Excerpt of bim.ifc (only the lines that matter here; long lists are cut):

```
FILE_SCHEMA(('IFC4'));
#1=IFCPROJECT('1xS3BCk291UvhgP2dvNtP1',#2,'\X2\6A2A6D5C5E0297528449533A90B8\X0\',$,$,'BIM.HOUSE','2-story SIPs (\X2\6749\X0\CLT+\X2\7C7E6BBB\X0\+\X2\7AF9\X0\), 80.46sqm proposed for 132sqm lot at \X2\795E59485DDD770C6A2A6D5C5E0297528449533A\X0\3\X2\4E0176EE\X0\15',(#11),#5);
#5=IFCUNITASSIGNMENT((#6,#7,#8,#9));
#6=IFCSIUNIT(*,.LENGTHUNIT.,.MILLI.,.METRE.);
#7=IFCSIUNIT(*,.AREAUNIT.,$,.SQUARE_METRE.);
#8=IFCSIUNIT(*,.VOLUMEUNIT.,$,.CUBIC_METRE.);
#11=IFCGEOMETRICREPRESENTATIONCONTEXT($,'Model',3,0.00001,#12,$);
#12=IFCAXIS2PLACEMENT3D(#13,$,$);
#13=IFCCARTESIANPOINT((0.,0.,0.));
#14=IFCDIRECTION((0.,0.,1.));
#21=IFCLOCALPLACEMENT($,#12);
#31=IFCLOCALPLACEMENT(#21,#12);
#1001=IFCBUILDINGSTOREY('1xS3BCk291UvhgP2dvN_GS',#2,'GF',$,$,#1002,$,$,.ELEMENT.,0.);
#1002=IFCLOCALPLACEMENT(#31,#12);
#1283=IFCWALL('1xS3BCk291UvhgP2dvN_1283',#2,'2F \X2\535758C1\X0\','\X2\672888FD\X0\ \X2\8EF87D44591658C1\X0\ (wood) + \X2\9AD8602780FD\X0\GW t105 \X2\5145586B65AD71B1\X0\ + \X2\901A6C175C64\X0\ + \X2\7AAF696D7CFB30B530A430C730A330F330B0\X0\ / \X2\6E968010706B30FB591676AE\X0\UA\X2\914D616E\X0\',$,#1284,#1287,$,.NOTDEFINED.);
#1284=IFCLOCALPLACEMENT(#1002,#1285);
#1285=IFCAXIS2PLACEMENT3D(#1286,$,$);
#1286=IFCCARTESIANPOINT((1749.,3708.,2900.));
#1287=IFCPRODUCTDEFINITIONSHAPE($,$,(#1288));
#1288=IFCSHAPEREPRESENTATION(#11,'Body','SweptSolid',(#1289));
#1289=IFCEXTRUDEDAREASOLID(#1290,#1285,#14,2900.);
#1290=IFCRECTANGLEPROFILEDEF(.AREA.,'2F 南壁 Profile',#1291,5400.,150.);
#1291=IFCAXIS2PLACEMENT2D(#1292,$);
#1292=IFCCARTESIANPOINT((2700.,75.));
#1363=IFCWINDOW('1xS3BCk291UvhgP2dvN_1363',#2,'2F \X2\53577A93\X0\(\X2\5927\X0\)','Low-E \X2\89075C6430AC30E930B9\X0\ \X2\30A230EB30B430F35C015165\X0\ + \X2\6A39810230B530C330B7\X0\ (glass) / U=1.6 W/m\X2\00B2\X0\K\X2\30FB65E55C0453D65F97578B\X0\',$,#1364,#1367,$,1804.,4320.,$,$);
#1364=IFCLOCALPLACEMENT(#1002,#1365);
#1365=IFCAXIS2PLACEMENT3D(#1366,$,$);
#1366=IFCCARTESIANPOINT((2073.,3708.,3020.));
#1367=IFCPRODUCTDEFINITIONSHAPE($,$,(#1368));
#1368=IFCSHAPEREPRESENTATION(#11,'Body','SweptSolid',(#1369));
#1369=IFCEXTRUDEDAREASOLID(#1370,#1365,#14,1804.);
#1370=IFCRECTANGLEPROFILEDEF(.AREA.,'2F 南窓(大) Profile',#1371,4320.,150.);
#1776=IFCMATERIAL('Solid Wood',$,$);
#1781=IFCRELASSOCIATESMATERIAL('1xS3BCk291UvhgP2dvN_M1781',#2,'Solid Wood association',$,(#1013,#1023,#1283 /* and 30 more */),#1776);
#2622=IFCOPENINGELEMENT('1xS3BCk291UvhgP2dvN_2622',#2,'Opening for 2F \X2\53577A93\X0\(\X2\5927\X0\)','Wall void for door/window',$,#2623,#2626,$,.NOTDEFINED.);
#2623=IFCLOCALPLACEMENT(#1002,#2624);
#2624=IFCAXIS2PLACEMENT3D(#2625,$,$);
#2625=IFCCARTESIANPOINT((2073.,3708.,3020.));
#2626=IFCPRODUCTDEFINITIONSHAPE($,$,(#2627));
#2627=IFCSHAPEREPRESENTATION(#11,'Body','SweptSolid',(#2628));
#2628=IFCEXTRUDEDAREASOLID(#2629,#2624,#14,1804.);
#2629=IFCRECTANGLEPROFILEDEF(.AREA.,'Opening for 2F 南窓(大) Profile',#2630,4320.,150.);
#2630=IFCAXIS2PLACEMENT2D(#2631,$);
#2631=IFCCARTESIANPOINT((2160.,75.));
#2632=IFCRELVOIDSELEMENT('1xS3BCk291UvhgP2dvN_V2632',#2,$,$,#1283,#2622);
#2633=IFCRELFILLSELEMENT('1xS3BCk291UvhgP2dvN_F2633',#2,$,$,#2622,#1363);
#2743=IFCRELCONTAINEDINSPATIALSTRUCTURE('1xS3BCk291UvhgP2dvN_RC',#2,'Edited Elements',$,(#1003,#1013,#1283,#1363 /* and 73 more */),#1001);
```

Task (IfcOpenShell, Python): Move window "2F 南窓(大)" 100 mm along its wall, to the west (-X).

```python
import ifcopenshell
import ifcopenshell.api.geometry
import ifcopenshell.util.placement

model = ifcopenshell.open("bim.ifc")

window = model.by_guid("1xS3BCk291UvhgP2dvN_1363")
opening = window.FillsVoids[0].RelatingOpeningElement
wall = opening.VoidsElements[0].RelatingBuildingElement

wall_matrix = ifcopenshell.util.placement.get_local_placement(wall.ObjectPlacement)
shift = wall_matrix[:3, 0] * -100.0
before = ifcopenshell.util.placement.get_local_placement(window.ObjectPlacement)[:3, 3].copy()

# The window is not placed relative to its opening, so move both.
for product in (opening, window):
    matrix = ifcopenshell.util.placement.get_local_placement(product.ObjectPlacement)
    matrix[:3, 3] += shift
    ifcopenshell.api.geometry.edit_object_placement(model, product=product, matrix=matrix, is_si=False)

after = ifcopenshell.util.placement.get_local_placement(window.ObjectPlacement)[:3, 3]
print("window moved by", (after - before).round(3) + 0.0)

model.write("bim-out.ifc")
```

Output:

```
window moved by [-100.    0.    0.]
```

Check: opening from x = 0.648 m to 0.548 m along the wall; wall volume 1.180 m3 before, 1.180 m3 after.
